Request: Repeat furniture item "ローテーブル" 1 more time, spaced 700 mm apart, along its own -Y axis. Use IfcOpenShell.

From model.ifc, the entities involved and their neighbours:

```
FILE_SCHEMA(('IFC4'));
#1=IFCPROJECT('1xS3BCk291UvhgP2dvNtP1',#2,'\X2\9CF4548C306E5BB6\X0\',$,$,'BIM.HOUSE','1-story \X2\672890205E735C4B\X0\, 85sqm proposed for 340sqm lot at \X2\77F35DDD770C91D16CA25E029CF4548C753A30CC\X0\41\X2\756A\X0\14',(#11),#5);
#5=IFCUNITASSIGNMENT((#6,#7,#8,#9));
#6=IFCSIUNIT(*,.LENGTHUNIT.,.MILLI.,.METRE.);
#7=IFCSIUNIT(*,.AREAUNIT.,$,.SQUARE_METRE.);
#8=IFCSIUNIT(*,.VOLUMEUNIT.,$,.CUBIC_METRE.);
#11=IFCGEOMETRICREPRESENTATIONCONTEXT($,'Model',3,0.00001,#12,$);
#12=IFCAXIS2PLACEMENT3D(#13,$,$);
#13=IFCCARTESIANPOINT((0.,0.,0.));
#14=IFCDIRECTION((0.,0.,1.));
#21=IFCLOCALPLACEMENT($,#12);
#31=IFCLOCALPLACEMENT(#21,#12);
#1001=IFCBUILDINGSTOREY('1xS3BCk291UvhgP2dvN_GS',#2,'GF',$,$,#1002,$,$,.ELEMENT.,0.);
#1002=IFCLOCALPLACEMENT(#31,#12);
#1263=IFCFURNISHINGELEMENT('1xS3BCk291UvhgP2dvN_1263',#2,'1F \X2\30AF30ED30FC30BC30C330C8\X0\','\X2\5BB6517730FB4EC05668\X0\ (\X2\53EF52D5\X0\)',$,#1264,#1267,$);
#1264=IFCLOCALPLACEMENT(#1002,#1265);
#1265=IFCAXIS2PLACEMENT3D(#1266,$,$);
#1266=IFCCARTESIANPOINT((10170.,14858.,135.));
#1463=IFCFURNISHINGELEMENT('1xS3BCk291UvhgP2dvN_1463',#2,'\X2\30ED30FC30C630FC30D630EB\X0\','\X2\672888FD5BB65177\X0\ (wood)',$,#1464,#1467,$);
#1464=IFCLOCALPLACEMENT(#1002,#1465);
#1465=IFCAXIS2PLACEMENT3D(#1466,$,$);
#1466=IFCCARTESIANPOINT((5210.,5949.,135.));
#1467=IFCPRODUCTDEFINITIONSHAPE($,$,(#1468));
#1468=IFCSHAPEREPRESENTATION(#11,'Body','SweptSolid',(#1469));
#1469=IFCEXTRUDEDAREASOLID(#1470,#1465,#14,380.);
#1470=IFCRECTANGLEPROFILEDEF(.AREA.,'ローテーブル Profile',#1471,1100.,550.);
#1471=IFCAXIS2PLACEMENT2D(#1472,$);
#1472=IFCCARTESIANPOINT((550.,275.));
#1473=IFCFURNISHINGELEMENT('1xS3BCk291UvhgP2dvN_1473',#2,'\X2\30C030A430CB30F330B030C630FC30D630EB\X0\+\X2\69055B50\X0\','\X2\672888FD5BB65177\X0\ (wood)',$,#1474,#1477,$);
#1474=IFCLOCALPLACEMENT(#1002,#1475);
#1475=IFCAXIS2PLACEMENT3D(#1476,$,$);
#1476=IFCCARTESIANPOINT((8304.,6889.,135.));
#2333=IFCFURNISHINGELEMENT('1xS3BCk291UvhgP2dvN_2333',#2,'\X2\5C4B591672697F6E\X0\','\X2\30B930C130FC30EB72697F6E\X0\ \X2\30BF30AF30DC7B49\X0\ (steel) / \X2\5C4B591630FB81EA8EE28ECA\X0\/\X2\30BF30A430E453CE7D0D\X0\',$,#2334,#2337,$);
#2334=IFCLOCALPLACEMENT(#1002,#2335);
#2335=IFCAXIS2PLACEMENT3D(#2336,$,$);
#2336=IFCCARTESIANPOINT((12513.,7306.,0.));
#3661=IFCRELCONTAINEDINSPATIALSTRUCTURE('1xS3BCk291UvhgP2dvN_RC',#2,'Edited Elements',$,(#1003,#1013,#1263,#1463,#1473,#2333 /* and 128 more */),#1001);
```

```python
import ifcopenshell
import ifcopenshell.api.geometry
import ifcopenshell.api.root
import ifcopenshell.util.element
import ifcopenshell.util.placement
import ifcopenshell.util.unit

model = ifcopenshell.open("model.ifc")
unit_scale = ifcopenshell.util.unit.calculate_unit_scale(model)


def reuse_history(source, copy):
    """copy_class also copies each property set's owner history, people and application; keep the originals."""
    for rel in copy.IsDefinedBy:
        if rel.is_a("IfcRelDefinesByProperties") and (history := rel.RelatingPropertyDefinition.OwnerHistory):
            rel.RelatingPropertyDefinition.OwnerHistory = source.OwnerHistory
            ifcopenshell.util.element.remove_deep2(model, history)


source = model.by_guid("1xS3BCk291UvhgP2dvN_1463")
base = ifcopenshell.util.placement.get_local_placement(source.ObjectPlacement)
step = -base[:3, 1] * 0.7 / unit_scale

for i in range(1, 2):
    copy = ifcopenshell.api.root.copy_class(model, product=source)
    copy.Representation = ifcopenshell.util.element.copy_deep(
        model, source.Representation, exclude=["IfcGeometricRepresentationContext", "IfcRepresentationMap"]
    )
    reuse_history(source, copy)
    matrix = base.copy()
    matrix[:3, 3] += i * step
    print("added at", matrix[:3, 3].round(3) + 0.0)
    ifcopenshell.api.geometry.edit_object_placement(model, product=copy, matrix=matrix, is_si=False)

model.write("model_updated.ifc")
```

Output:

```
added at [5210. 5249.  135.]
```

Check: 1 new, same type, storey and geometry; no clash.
